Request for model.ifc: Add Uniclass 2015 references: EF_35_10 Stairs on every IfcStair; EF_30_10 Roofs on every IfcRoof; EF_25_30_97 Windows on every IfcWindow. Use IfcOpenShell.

First a look at what the model holds.

```python
import ifcopenshell

model = ifcopenshell.open("model.ifc")
print(model.schema)
print("classifications:", [c.Name for c in model.by_type("IfcClassification")])
for ifc_class in ("IfcDoor", "IfcRoof", "IfcStair", "IfcWall", "IfcWindow"):
    print(ifc_class, len(model.by_type(ifc_class)))
```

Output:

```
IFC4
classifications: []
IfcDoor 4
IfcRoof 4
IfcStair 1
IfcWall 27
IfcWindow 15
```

```python
import ifcopenshell
import ifcopenshell.api.classification

model = ifcopenshell.open("model.ifc")

system = ifcopenshell.api.classification.add_classification(model, classification="Uniclass 2015")

codes = {
    "IfcStair": ("EF_35_10", "Stairs"),
    "IfcRoof": ("EF_30_10", "Roofs"),
    "IfcWindow": ("EF_25_30_97", "Windows"),
}
for ifc_class, (code, name) in codes.items():
    products = model.by_type(ifc_class)
    ifcopenshell.api.classification.add_reference(
        model, products=products, classification=system, identification=code, name=name
    )
    print(code, len(products))

model.write("model_edited.ifc")
```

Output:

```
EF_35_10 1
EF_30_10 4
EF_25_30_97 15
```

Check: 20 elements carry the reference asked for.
